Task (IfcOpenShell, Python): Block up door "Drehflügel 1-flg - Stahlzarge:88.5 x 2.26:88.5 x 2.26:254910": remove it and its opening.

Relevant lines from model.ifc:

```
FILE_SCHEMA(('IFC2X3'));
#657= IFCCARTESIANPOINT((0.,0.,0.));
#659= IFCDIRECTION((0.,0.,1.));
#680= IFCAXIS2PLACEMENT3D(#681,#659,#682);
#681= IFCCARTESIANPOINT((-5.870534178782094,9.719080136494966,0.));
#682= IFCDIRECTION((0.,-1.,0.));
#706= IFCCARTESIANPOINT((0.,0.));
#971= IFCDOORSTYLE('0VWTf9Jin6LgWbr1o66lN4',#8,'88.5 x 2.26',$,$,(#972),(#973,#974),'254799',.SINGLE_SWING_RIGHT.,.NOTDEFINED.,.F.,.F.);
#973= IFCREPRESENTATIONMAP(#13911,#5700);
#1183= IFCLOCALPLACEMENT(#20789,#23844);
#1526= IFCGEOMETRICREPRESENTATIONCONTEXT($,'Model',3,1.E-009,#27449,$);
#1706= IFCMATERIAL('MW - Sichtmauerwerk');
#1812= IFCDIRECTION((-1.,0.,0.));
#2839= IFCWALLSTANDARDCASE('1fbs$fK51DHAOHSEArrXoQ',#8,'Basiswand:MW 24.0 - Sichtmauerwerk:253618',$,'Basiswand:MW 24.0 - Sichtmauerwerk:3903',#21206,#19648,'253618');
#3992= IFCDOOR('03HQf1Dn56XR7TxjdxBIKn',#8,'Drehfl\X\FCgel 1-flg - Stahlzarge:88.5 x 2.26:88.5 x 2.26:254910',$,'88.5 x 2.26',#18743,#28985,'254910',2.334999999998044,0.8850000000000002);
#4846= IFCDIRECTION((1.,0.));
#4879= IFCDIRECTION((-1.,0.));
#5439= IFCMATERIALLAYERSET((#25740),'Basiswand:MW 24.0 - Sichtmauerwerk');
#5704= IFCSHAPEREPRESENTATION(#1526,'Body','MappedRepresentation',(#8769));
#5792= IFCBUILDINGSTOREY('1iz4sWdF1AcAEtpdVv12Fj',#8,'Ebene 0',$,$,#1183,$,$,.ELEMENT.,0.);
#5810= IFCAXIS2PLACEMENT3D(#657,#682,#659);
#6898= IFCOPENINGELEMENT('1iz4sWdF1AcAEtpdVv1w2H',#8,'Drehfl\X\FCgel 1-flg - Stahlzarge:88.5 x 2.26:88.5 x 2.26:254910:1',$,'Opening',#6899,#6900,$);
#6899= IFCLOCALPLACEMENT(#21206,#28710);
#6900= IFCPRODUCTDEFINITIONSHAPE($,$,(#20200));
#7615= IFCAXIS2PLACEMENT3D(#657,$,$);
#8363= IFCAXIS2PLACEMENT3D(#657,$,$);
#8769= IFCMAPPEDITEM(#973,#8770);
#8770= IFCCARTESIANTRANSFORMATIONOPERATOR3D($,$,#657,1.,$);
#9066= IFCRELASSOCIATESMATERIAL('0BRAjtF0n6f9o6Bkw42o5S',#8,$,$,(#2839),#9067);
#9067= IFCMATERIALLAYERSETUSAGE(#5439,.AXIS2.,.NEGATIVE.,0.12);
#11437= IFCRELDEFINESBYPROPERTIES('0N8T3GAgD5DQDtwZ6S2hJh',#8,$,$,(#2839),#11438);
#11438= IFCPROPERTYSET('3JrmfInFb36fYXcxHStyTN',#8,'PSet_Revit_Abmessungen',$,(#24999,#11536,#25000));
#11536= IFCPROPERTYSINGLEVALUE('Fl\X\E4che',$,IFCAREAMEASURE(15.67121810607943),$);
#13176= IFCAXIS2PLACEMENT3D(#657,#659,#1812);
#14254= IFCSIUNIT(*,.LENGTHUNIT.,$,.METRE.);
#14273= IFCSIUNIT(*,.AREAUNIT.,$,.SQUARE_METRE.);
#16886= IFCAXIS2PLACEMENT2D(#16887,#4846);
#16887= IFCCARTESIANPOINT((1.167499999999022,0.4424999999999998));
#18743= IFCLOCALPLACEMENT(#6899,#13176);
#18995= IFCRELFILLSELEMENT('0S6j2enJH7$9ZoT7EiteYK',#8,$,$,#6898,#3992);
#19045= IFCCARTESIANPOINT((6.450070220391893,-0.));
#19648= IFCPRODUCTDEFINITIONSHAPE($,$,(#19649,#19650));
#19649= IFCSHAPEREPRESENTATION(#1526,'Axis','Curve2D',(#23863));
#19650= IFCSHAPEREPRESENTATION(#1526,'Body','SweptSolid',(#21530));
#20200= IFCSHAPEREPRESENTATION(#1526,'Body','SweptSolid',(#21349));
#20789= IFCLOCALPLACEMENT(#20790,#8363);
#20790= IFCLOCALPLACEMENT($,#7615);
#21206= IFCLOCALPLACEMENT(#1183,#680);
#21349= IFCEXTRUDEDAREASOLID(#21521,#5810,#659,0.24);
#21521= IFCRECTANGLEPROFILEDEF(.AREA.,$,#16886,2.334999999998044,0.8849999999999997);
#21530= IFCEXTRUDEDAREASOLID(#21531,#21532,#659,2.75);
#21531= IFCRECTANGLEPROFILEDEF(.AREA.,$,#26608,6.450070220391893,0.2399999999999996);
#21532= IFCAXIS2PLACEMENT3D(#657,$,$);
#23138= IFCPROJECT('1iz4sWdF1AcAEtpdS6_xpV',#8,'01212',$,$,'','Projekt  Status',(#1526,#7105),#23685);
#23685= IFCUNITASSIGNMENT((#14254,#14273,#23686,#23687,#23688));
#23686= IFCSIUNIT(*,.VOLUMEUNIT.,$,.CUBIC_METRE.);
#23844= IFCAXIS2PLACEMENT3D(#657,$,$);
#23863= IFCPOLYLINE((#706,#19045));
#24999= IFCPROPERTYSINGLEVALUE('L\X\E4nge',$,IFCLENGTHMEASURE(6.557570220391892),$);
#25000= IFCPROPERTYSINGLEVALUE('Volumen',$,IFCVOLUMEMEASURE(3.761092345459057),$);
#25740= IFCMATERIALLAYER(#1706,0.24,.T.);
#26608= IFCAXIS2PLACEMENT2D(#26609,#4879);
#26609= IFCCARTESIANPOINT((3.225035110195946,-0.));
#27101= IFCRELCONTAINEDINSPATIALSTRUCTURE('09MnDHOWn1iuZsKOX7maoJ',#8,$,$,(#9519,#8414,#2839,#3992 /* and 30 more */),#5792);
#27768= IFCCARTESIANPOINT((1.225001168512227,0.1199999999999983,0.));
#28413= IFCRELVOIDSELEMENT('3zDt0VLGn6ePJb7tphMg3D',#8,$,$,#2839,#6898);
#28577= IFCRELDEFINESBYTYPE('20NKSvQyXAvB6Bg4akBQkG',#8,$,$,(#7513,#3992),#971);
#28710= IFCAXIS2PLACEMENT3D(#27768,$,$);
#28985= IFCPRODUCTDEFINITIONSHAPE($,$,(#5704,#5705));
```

```python
import ifcopenshell
import ifcopenshell.api.feature
import ifcopenshell.api.pset
import ifcopenshell.api.root
import ifcopenshell.geom
import ifcopenshell.util.element
import ifcopenshell.util.shape
import ifcopenshell.util.unit

model = ifcopenshell.open("model.ifc")
area_scale = ifcopenshell.util.unit.calculate_unit_scale(model, "AREAUNIT")
volume_scale = ifcopenshell.util.unit.calculate_unit_scale(model, "VOLUMEUNIT")
settings = ifcopenshell.geom.settings()


def volume(element):
    """Net volume in cubic metres, openings subtracted."""
    shape = ifcopenshell.geom.create_shape(settings, element)
    return ifcopenshell.util.shape.get_volume(shape.geometry)


door = model.by_guid("03HQf1Dn56XR7TxjdxBIKn")
opening = door.FillsVoids[0].RelatingOpeningElement
wall = opening.VoidsElements[0].RelatingBuildingElement
before = volume(wall)

ifcopenshell.api.root.remove_product(model, product=door)
ifcopenshell.api.feature.remove_feature(model, feature=opening)

after = volume(wall)
thickness = 0.24  # wall thickness in metres

# Update the wall's stored quantities.
pset = model.by_id(ifcopenshell.util.element.get_pset(wall, "PSet_Revit_Abmessungen", should_inherit=False)["id"])
ifcopenshell.api.pset.edit_pset(model, pset=pset, properties={
    "Fläche": model.create_entity("IfcAreaMeasure", after / thickness / area_scale),
    "Volumen": model.create_entity("IfcVolumeMeasure", after / volume_scale),
})

print(f"wall volume {before:.3f} -> {after:.3f} m3")

model.write("model_edited.ifc")
```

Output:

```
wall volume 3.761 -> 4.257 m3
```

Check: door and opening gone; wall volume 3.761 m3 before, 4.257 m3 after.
